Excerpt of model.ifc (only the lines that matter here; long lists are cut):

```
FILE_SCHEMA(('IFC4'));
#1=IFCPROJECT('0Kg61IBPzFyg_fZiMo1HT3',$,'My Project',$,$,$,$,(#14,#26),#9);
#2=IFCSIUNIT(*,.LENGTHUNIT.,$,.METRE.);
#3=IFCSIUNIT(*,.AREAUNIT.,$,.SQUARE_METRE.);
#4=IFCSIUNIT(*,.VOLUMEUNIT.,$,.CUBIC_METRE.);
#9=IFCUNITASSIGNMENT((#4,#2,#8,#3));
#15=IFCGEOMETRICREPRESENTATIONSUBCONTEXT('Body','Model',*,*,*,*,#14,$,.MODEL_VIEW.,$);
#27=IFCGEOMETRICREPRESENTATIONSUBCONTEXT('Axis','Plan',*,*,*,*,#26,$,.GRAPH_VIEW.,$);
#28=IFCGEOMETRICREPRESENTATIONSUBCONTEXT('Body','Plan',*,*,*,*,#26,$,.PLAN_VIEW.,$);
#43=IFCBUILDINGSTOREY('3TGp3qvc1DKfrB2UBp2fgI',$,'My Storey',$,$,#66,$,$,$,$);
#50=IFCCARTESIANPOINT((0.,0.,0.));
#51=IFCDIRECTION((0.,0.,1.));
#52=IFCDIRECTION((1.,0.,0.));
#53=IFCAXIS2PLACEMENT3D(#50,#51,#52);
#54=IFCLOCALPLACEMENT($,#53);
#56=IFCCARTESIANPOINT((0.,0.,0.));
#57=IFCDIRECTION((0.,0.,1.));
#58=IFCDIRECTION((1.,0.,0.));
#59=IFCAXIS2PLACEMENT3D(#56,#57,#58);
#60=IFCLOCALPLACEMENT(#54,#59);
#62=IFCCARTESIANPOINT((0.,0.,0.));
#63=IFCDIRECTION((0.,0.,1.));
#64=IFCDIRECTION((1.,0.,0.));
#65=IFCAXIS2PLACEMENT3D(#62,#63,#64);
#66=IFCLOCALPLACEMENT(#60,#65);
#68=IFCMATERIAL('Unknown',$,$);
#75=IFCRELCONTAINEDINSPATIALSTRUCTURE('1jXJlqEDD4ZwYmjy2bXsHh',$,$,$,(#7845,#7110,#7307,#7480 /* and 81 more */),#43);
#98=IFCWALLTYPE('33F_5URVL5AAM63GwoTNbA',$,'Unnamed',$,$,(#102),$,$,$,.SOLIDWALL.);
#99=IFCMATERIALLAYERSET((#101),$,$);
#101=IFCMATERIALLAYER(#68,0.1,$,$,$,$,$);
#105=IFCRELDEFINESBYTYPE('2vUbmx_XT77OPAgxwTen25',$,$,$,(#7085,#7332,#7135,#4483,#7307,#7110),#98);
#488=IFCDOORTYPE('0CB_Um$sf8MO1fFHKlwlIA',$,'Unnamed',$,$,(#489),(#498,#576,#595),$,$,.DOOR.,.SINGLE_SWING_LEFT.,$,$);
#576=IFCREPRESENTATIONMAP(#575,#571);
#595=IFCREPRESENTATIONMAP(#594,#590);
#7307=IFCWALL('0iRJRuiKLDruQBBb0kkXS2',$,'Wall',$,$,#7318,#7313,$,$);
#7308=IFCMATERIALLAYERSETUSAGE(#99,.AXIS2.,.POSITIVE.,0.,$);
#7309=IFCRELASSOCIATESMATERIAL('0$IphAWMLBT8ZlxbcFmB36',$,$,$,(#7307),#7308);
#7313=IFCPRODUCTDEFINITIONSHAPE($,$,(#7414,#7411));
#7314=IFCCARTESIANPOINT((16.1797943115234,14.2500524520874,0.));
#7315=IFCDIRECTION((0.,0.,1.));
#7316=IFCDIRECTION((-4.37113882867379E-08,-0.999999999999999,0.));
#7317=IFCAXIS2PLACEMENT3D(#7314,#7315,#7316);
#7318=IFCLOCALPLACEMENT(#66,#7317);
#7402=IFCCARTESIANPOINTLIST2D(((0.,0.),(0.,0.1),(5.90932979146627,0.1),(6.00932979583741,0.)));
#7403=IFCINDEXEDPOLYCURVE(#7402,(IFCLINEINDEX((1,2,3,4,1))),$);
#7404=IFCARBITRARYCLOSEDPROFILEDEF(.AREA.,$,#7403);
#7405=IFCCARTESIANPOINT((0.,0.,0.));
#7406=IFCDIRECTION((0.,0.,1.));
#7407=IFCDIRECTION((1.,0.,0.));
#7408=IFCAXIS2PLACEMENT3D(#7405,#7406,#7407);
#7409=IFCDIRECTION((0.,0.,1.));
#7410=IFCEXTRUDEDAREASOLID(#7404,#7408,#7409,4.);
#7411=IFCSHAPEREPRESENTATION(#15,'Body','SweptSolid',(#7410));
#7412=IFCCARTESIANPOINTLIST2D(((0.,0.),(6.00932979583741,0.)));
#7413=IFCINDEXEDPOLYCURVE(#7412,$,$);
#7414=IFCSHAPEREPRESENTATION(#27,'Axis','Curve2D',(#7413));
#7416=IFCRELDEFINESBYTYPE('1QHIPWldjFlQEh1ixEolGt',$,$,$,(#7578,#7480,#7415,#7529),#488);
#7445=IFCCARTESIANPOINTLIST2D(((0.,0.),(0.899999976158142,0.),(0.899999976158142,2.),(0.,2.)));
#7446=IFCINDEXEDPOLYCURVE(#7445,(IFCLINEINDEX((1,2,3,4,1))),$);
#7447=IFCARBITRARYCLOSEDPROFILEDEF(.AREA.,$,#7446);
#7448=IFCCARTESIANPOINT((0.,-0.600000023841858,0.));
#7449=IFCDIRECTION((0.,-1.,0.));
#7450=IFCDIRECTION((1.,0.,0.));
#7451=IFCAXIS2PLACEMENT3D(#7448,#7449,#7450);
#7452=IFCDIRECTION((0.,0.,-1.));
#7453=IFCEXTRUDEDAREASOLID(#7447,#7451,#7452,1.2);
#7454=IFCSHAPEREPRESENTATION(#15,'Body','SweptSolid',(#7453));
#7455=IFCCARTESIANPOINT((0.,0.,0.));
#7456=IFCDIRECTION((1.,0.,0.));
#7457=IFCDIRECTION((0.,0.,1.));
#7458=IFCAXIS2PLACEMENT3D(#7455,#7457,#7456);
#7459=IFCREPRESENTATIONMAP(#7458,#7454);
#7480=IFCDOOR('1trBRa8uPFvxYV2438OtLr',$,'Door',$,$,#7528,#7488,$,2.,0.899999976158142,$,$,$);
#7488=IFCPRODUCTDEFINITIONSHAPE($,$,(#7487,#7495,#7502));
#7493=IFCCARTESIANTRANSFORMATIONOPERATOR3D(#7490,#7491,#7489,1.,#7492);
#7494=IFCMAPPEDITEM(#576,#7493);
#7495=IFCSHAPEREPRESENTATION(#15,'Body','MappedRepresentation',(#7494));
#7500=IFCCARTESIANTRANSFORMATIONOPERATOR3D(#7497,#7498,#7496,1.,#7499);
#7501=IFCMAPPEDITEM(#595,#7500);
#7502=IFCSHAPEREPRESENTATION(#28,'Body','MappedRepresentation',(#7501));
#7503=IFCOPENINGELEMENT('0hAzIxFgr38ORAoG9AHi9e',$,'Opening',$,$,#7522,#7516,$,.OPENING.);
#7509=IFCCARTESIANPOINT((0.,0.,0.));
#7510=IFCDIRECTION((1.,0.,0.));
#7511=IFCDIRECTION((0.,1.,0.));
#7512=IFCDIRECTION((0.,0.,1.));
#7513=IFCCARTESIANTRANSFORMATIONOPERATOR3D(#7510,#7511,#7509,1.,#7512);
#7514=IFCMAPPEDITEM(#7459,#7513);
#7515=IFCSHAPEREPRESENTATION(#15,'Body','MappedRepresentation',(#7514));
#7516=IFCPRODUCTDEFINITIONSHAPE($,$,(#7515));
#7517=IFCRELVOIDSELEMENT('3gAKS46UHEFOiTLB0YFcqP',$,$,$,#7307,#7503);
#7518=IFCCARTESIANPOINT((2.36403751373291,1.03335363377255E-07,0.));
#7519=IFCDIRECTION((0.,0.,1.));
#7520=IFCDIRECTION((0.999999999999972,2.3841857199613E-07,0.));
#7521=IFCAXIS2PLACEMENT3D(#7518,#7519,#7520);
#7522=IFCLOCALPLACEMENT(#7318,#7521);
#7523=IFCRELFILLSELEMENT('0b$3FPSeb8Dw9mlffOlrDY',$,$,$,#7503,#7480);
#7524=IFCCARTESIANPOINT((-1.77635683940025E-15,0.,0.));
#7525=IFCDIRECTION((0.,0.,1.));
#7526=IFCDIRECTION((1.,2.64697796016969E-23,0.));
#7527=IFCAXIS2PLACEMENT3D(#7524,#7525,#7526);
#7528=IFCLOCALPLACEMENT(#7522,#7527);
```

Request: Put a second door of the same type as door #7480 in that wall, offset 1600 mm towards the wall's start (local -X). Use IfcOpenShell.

```python
import ifcopenshell
import ifcopenshell.api.feature
import ifcopenshell.api.geometry
import ifcopenshell.api.root
import ifcopenshell.geom
import ifcopenshell.util.element
import ifcopenshell.util.placement
import ifcopenshell.util.shape

model = ifcopenshell.open("model.ifc")
settings = ifcopenshell.geom.settings()


def volume(element):
    """Net volume in cubic metres, openings subtracted."""
    shape = ifcopenshell.geom.create_shape(settings, element)
    return ifcopenshell.util.shape.get_volume(shape.geometry)


door = model.by_id(7480)
opening = door.FillsVoids[0].RelatingOpeningElement
wall = opening.VoidsElements[0].RelatingBuildingElement
before = volume(wall)
shift = ifcopenshell.util.placement.get_local_placement(wall.ObjectPlacement)[:3, 0] * -1.6

# copy_class copies the void relationship, type, container and properties, but no geometry.
new_opening = ifcopenshell.api.root.copy_class(model, product=opening)
new_opening.Representation = ifcopenshell.util.element.copy_deep(
    model, opening.Representation, exclude=["IfcGeometricRepresentationContext", "IfcRepresentationMap"]
)
new_door = ifcopenshell.api.root.copy_class(model, product=door)
new_door.Representation = ifcopenshell.util.element.copy_deep(
    model, door.Representation, exclude=["IfcGeometricRepresentationContext", "IfcRepresentationMap"]
)
ifcopenshell.api.feature.add_filling(model, opening=new_opening, element=new_door)

for old, new in ((opening, new_opening), (door, new_door)):
    matrix = ifcopenshell.util.placement.get_local_placement(old.ObjectPlacement)
    matrix[:3, 3] += shift
    ifcopenshell.api.geometry.edit_object_placement(model, product=new, matrix=matrix, is_si=False)

after = volume(wall)

print(f"wall volume {before:.3f} -> {after:.3f} m3")

model.write("model_v2.ifc")
```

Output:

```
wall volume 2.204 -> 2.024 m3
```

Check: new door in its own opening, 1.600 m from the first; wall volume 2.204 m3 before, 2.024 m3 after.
